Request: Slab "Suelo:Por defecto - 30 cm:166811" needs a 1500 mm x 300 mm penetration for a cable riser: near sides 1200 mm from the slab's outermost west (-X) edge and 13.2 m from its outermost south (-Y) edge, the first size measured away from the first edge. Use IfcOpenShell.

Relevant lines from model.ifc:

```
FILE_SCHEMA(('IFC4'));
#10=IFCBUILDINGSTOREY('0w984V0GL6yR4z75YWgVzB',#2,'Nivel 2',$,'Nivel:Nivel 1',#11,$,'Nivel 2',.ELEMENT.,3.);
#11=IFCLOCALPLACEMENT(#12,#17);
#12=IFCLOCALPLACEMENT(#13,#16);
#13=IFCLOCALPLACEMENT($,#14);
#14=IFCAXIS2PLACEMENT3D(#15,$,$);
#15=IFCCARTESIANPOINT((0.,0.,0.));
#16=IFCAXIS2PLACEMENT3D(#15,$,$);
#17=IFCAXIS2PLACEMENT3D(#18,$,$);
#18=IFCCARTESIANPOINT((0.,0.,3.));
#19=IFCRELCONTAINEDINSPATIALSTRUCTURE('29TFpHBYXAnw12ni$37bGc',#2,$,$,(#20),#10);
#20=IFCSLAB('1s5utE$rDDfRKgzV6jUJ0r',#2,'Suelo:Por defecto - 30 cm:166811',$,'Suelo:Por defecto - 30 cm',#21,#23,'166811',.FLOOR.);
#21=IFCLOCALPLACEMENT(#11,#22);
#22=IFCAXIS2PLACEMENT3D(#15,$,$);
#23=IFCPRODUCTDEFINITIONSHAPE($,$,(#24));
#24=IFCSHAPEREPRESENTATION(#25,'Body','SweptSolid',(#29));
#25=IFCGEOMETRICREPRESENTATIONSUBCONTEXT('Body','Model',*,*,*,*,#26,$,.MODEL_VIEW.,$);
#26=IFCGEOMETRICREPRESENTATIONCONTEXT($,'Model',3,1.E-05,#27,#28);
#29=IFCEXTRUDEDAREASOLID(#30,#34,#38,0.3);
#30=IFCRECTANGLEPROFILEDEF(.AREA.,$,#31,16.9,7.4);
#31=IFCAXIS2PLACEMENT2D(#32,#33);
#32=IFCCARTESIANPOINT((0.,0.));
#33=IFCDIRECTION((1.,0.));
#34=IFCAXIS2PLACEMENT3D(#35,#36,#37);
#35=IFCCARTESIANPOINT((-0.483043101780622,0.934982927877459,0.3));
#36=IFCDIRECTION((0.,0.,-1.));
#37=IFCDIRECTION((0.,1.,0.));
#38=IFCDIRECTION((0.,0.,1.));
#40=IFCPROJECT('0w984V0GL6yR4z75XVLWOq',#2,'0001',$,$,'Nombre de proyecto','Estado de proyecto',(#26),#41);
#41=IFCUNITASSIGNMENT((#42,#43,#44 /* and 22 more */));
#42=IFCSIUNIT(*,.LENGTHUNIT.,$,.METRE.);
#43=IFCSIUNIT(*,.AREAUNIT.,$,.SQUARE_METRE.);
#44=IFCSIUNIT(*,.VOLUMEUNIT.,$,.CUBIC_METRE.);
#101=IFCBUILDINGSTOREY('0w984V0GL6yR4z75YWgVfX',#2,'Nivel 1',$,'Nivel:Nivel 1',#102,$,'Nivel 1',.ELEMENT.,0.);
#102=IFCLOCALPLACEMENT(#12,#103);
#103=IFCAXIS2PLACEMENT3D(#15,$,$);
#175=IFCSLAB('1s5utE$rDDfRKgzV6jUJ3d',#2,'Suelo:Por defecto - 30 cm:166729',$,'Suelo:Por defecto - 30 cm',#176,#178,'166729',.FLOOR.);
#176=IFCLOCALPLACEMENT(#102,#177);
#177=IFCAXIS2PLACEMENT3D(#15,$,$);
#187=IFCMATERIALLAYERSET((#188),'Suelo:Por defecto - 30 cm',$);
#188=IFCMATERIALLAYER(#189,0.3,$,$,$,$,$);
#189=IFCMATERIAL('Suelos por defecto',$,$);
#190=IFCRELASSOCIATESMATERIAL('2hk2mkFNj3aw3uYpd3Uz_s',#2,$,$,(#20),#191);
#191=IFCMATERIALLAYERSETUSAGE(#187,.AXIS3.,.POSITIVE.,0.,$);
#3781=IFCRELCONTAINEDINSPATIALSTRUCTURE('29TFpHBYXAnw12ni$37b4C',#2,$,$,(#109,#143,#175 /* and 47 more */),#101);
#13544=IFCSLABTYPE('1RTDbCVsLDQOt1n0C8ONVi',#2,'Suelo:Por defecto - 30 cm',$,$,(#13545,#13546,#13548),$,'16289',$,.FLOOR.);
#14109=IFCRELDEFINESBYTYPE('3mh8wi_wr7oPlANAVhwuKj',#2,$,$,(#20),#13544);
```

```python
import numpy as np
import ifcopenshell
import ifcopenshell.api.feature
import ifcopenshell.api.geometry
import ifcopenshell.api.root
import ifcopenshell.geom
import ifcopenshell.util.placement
import ifcopenshell.util.representation
import ifcopenshell.util.shape
import ifcopenshell.util.unit

model = ifcopenshell.open("model.ifc")
unit_scale = ifcopenshell.util.unit.calculate_unit_scale(model)
settings = ifcopenshell.geom.settings()


def volume(element):
    """Net volume in cubic metres, openings subtracted."""
    shape = ifcopenshell.geom.create_shape(settings, element)
    return ifcopenshell.util.shape.get_volume(shape.geometry)


slab = model.by_guid("1s5utE$rDDfRKgzV6jUJ0r")
before = volume(slab)

# Extent in the slab's own axes, in metres. The edges named are its -X and -Y sides.
slab_shape = ifcopenshell.geom.create_shape(settings, slab)
vertices = ifcopenshell.util.shape.get_vertices(slab_shape.geometry)
x_min, y_min, bottom = vertices.min(axis=0)
top = vertices[:, 2].max()

opening = ifcopenshell.api.root.create_entity(model, ifc_class="IfcOpeningElement", name="Cable riser opening", predefined_type="OPENING")
context = ifcopenshell.util.representation.get_context(model, "Model", "Body", "MODEL_VIEW")
width, depth = 1.5, 0.3
outline = [(0.0, 0.0), (width, 0.0), (width, depth), (0.0, depth), (0.0, 0.0)]
# Overshoot both faces by 50 mm so the cut is clean.
shape = ifcopenshell.api.geometry.add_slab_representation(
    model, context=context, depth=top - bottom + 0.1, polyline=outline
)
ifcopenshell.api.geometry.assign_representation(model, product=opening, representation=shape)

matrix = ifcopenshell.util.placement.get_local_placement(slab.ObjectPlacement)
matrix[:, 3] = matrix @ np.append(np.array([x_min + 1.2, y_min + 13.2, bottom - 0.05]) / unit_scale, 1.0)
ifcopenshell.api.geometry.edit_object_placement(model, product=opening, matrix=matrix, is_si=False)
ifcopenshell.api.feature.add_feature(model, feature=opening, element=slab)

after = volume(slab)

print(f"slab volume {before:.3f} -> {after:.3f} m3")

model.write("model_rev.ifc")
```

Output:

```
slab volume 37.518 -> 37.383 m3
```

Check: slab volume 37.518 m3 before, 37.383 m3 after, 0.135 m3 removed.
